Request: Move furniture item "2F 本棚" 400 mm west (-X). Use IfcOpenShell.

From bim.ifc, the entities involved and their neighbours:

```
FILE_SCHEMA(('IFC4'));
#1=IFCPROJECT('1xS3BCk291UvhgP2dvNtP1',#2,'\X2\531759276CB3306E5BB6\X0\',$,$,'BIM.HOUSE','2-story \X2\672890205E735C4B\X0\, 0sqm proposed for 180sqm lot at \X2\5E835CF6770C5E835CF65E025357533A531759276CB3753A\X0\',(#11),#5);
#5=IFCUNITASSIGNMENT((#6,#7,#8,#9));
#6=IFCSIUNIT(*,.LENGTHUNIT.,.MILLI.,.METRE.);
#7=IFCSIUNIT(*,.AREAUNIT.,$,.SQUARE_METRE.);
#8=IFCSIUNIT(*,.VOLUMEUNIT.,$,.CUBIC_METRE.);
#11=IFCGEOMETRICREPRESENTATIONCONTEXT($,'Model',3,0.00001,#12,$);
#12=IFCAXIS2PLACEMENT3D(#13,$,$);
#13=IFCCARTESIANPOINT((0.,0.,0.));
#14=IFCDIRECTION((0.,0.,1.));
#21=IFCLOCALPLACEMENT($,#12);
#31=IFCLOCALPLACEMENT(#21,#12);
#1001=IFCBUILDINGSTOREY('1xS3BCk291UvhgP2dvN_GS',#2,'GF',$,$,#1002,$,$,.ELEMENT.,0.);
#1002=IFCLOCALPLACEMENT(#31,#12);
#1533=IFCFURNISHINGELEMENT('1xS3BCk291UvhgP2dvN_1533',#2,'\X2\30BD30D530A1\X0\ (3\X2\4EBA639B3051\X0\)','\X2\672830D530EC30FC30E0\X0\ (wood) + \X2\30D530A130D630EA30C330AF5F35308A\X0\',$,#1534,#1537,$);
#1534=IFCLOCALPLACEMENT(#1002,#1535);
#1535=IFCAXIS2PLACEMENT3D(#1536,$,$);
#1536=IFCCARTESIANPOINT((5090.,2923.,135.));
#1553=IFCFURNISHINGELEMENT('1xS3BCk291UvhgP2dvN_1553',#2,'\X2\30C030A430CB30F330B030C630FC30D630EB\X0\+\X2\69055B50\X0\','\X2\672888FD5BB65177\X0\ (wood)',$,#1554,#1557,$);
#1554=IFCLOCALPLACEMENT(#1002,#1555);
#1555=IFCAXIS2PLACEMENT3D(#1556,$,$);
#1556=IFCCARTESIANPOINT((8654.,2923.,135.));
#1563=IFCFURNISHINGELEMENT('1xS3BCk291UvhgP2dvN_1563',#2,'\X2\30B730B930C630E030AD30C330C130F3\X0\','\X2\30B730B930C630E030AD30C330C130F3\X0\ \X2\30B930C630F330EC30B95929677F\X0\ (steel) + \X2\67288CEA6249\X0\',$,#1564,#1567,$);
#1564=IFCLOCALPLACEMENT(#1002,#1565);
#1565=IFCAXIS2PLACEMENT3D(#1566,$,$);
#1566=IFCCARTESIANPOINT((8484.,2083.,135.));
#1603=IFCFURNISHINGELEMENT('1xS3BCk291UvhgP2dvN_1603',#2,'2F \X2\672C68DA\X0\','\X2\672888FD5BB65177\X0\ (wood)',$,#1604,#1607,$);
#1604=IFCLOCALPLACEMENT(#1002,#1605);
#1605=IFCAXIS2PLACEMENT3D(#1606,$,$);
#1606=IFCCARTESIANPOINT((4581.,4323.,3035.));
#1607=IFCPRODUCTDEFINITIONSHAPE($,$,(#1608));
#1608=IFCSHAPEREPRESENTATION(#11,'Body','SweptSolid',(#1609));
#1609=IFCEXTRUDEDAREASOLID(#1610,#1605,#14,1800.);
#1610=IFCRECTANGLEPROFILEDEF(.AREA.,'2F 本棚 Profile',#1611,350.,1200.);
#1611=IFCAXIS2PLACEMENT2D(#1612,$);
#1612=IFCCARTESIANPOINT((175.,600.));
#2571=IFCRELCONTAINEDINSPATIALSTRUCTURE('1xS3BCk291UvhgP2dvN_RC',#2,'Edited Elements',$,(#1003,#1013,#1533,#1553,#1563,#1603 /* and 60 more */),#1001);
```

```python
import ifcopenshell
import ifcopenshell.api.geometry
import ifcopenshell.util.placement
import ifcopenshell.util.unit

model = ifcopenshell.open("bim.ifc")
unit_scale = ifcopenshell.util.unit.calculate_unit_scale(model)

item = model.by_id(1603)
matrix = ifcopenshell.util.placement.get_local_placement(item.ObjectPlacement)
matrix[0, 3] -= 0.4 / unit_scale
ifcopenshell.api.geometry.edit_object_placement(model, product=item, matrix=matrix, is_si=False)

print(ifcopenshell.util.placement.get_local_placement(item.ObjectPlacement).round(3) + 0.0)

model.write("bim_rev.ifc")
```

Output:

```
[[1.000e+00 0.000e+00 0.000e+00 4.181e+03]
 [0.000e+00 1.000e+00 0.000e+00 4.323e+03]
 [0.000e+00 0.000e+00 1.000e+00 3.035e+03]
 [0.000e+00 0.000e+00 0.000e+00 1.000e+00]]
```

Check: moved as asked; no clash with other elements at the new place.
